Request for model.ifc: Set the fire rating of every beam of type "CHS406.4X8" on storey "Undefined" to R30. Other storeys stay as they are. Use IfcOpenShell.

First a look at what the model holds.

```python
import ifcopenshell
import ifcopenshell.util.element

model = ifcopenshell.open("model.ifc")
print(model.schema)
storey = next(s for s in model.by_type("IfcBuildingStorey") if s.Name == "Undefined")
beams = [e for e in ifcopenshell.util.element.get_decomposition(storey) if e.is_a("IfcBeam")]
seen = {}
for e in beams:
    element_type = ifcopenshell.util.element.get_type(e)
    key = (element_type.Name if element_type != e and element_type else None, ifcopenshell.util.element.get_pset(e, "Pset_BeamCommon", "FireRating"))
    seen[key] = seen.get(key, 0) + 1
for (name, value), count in sorted(seen.items(), key=str):
    print(count, "x", name, "|", value)
```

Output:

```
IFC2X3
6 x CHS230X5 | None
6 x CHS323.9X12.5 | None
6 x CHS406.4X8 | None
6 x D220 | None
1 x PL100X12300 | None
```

```python
import ifcopenshell
import ifcopenshell.api.pset
import ifcopenshell.util.element

model = ifcopenshell.open("model.ifc")

storey = next(s for s in model.by_type("IfcBuildingStorey") if s.Name == "Undefined")
beams = [e for e in ifcopenshell.util.element.get_decomposition(storey) if e.is_a("IfcBeam")]

count = 0
for e in beams:
    element_type = ifcopenshell.util.element.get_type(e)
    if element_type in (None, e) or element_type.Name != "CHS406.4X8":
        continue
    found = ifcopenshell.util.element.get_pset(e, "Pset_BeamCommon", should_inherit=False)
    if found:
        pset = model.by_id(found["id"])
        if len(ifcopenshell.util.element.get_elements_by_pset(pset)) > 1:
            pset = ifcopenshell.api.pset.unshare_pset(model, products=[e], pset=pset)[0]
    else:
        pset = ifcopenshell.api.pset.add_pset(model, product=e, name="Pset_BeamCommon")
    ifcopenshell.api.pset.edit_pset(model, pset=pset, properties={"FireRating": "R30"})
    count += 1

print(count, "beams updated")

model.write("model_updated.ifc")
```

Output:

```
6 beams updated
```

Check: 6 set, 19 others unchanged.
